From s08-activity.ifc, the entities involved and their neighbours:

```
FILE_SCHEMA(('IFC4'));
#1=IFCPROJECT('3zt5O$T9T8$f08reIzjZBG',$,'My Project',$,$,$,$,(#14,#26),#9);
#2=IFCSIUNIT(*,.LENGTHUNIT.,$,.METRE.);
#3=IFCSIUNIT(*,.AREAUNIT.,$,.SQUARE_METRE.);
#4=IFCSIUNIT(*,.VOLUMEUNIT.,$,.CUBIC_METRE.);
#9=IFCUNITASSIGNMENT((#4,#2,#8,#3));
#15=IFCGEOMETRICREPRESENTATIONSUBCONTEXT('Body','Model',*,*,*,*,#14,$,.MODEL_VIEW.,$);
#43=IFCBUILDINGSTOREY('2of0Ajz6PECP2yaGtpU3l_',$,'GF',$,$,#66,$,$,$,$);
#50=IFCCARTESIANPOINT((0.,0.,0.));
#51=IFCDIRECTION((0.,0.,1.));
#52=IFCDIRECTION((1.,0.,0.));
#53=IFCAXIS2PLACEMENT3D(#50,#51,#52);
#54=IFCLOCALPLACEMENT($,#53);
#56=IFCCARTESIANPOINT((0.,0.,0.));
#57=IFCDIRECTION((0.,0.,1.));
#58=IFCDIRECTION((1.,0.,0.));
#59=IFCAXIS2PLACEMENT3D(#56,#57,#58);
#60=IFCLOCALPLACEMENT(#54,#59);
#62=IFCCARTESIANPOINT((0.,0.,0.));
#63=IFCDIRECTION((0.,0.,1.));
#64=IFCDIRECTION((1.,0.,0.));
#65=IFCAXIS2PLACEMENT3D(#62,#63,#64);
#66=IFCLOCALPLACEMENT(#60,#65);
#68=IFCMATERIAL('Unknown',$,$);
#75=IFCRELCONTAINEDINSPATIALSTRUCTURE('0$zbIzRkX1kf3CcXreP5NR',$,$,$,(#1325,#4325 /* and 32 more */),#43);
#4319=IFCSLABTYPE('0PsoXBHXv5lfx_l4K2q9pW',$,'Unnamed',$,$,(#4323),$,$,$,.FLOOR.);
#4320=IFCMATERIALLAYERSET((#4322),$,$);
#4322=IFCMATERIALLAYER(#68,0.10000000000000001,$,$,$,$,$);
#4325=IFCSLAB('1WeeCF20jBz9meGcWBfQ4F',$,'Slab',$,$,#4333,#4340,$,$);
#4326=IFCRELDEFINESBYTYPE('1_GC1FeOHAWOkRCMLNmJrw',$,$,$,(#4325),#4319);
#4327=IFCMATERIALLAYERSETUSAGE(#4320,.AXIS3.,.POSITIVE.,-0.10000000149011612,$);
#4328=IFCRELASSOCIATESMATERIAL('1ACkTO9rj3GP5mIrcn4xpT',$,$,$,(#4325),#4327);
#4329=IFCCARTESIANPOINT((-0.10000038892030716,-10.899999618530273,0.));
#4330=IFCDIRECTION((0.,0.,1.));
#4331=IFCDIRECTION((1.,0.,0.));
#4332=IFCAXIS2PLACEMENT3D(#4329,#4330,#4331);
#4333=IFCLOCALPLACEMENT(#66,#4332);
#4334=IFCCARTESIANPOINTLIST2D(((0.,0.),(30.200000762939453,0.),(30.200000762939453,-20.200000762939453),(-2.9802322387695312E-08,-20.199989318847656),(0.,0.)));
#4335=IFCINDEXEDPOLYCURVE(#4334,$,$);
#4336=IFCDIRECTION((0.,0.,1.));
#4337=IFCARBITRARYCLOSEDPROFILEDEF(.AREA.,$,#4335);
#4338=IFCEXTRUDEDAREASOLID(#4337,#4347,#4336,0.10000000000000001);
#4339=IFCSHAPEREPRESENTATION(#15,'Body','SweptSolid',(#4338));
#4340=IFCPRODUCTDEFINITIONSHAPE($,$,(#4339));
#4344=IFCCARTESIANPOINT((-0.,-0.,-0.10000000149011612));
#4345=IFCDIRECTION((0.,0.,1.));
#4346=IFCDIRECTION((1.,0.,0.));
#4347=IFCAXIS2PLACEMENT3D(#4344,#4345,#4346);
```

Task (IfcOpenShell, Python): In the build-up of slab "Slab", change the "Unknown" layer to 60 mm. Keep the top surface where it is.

```python
import ifcopenshell
import ifcopenshell.util.element
import ifcopenshell.util.representation
import ifcopenshell.util.unit

model = ifcopenshell.open("s08-activity.ifc")
unit_scale = ifcopenshell.util.unit.calculate_unit_scale(model)

layer_set = model.by_id(4320)
layer = next(l for l in layer_set.MaterialLayers if l.Material and l.Material.Name == "Unknown")
change = 0.06 / unit_scale - layer.LayerThickness
layer.LayerThickness += change

# Geometry does not follow the layer set by itself.
slabs = [e for e in ifcopenshell.util.element.get_elements_by_material(model, layer_set) if e.is_a("IfcSlab")]
for slab in sorted(slabs, key=lambda e: e.id()):
    body = ifcopenshell.util.representation.get_representation(slab, "Model", "Body")
    solid = body.Items[0]
    old_depth = solid.Depth
    solid.Depth += change
    # Extruded upwards: lower the start of the extrusion so the top stays.
    x, y, z = solid.Position.Location.Coordinates
    solid.Position.Location = model.createIfcCartesianPoint((x, y, z - change))
    print(slab.id(), f"{old_depth:g} -> {solid.Depth:g}")

# The layers are counted up from the underside, which has moved.
for usage in {ifcopenshell.util.element.get_material(slab) for slab in slabs}:
    usage.OffsetFromReferenceLine -= change

model.write("s08-activity_v2.ifc")
```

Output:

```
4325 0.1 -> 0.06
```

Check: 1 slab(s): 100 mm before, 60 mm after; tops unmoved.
